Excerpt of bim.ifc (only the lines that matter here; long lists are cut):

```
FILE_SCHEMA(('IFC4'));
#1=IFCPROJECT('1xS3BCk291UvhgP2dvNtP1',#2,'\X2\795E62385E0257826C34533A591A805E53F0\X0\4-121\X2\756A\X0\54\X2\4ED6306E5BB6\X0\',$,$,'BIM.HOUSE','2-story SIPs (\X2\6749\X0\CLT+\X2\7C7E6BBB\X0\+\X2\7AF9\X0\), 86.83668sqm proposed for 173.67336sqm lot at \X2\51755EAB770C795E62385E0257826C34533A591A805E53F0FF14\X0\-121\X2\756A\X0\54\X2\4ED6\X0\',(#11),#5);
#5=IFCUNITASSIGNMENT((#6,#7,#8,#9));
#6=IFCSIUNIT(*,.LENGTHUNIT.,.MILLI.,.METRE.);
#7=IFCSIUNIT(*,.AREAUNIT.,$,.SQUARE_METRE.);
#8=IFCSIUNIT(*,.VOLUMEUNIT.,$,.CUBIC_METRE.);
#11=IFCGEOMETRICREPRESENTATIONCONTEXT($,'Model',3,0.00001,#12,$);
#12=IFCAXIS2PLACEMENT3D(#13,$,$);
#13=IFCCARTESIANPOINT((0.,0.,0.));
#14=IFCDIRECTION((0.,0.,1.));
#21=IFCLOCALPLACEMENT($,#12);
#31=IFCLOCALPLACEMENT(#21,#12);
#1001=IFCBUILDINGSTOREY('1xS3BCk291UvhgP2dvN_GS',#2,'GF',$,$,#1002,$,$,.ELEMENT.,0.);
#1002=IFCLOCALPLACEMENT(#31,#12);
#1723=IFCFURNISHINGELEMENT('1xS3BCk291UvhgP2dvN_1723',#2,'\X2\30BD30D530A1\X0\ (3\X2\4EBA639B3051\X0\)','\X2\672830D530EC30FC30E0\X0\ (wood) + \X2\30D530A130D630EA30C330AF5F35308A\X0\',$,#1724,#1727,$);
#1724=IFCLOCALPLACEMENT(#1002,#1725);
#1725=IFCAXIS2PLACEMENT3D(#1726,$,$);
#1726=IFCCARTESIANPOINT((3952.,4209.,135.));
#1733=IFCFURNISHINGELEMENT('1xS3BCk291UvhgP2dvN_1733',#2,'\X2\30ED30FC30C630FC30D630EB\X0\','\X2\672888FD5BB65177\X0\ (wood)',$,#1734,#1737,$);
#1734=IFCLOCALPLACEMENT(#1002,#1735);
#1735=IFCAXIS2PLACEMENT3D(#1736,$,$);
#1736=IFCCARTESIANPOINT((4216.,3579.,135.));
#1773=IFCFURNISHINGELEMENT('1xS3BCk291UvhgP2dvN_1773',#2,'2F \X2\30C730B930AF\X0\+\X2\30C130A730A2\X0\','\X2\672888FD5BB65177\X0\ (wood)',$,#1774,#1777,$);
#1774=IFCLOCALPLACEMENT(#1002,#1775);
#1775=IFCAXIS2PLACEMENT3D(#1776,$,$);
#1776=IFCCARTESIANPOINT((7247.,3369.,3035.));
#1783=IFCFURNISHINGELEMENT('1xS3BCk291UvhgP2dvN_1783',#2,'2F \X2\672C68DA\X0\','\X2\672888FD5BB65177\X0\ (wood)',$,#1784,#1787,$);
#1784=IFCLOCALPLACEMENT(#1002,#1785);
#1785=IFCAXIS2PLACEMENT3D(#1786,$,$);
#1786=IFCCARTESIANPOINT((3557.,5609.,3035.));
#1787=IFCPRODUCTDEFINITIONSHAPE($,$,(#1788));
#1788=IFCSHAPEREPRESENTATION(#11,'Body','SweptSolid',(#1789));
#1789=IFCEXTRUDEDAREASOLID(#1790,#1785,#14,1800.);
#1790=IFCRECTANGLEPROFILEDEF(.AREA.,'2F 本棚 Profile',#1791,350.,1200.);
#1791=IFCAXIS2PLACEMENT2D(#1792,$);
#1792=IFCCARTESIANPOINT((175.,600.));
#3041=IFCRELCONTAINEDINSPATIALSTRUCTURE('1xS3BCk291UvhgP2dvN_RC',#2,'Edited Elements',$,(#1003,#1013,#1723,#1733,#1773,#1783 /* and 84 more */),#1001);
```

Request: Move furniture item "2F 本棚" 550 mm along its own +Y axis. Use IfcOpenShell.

```python
import ifcopenshell
import ifcopenshell.api.geometry
import ifcopenshell.util.placement
import ifcopenshell.util.unit

model = ifcopenshell.open("bim.ifc")
unit_scale = ifcopenshell.util.unit.calculate_unit_scale(model)

item = model.by_id(1783)
matrix = ifcopenshell.util.placement.get_local_placement(item.ObjectPlacement)
matrix[:3, 3] += matrix[:3, 1] * 0.55 / unit_scale
ifcopenshell.api.geometry.edit_object_placement(model, product=item, matrix=matrix, is_si=False)

print(ifcopenshell.util.placement.get_local_placement(item.ObjectPlacement).round(3) + 0.0)

model.write("bim_v2.ifc")
```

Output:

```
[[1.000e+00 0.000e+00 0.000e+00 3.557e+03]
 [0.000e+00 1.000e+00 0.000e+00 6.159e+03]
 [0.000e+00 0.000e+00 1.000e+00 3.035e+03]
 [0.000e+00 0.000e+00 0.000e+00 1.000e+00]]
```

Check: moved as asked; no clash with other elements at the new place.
